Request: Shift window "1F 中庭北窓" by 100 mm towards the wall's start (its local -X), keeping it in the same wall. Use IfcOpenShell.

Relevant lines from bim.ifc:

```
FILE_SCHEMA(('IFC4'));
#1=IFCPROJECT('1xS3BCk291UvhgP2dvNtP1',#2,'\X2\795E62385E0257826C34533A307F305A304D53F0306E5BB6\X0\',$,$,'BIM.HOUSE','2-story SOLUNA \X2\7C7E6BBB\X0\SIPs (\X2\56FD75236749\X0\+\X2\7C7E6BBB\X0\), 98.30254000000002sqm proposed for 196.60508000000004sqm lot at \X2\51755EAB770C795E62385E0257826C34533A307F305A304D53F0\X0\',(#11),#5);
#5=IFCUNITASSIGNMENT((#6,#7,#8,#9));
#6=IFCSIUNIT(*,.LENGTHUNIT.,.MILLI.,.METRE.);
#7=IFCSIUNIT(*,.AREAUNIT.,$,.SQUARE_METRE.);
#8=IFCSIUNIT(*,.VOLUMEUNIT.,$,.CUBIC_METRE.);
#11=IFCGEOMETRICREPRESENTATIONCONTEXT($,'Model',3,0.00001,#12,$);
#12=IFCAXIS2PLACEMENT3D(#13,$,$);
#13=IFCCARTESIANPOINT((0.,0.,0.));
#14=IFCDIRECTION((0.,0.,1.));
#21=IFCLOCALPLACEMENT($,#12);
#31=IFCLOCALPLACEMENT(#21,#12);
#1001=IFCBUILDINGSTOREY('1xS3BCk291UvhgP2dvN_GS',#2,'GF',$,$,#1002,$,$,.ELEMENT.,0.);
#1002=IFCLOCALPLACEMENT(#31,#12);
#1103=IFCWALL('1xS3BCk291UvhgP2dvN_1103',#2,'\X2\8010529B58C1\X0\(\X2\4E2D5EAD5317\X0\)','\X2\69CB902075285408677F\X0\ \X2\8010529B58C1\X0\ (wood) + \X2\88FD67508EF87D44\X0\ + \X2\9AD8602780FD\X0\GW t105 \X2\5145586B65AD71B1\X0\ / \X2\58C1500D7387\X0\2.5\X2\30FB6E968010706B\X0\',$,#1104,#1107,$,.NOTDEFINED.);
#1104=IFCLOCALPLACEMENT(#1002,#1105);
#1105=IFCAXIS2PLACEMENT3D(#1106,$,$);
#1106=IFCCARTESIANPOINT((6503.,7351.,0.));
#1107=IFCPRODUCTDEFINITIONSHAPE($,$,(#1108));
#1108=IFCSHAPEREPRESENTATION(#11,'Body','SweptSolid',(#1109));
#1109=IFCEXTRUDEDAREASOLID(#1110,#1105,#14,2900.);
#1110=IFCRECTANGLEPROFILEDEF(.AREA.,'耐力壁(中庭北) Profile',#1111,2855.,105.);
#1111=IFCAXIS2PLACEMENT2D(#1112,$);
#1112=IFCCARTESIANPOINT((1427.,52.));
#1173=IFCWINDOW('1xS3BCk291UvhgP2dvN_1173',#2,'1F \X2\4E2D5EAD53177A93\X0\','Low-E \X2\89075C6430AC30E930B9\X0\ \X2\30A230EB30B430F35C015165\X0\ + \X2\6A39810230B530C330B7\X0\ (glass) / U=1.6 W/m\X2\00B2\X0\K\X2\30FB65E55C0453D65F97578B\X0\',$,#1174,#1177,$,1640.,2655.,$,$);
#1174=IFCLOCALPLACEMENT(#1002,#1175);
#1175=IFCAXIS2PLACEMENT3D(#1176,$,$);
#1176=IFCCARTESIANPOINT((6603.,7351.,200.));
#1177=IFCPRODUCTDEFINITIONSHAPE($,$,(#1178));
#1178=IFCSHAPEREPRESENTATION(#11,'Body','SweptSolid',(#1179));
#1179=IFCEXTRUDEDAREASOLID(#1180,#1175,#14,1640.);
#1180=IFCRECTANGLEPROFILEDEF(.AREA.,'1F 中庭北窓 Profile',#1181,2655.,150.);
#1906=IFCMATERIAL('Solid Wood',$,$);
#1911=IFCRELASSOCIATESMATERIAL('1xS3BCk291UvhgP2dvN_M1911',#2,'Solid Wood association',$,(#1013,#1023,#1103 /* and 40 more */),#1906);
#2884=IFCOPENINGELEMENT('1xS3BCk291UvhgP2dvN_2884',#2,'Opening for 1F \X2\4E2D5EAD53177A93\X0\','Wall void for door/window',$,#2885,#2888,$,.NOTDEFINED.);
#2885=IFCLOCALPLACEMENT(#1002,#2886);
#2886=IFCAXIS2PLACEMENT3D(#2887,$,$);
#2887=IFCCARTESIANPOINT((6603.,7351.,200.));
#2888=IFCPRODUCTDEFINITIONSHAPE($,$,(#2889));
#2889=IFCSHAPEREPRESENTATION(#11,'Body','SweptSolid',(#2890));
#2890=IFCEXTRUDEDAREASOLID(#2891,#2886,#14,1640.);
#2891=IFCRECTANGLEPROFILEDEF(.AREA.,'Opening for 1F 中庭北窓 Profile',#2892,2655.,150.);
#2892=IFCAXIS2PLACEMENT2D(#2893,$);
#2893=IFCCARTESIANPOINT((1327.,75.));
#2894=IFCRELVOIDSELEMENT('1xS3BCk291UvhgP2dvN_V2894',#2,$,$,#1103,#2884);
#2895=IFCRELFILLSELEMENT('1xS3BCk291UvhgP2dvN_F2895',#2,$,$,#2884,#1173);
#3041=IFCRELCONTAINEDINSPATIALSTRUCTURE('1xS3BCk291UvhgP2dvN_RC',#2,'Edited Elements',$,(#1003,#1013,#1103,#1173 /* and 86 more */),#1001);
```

```python
import ifcopenshell
import ifcopenshell.api.geometry
import ifcopenshell.util.placement

model = ifcopenshell.open("bim.ifc")

window = model.by_guid("1xS3BCk291UvhgP2dvN_1173")
opening = window.FillsVoids[0].RelatingOpeningElement
wall = opening.VoidsElements[0].RelatingBuildingElement

wall_matrix = ifcopenshell.util.placement.get_local_placement(wall.ObjectPlacement)
shift = wall_matrix[:3, 0] * -100.0
before = ifcopenshell.util.placement.get_local_placement(window.ObjectPlacement)[:3, 3].copy()

# The window is not placed relative to its opening, so move both.
for product in (opening, window):
    matrix = ifcopenshell.util.placement.get_local_placement(product.ObjectPlacement)
    matrix[:3, 3] += shift
    ifcopenshell.api.geometry.edit_object_placement(model, product=product, matrix=matrix, is_si=False)

after = ifcopenshell.util.placement.get_local_placement(window.ObjectPlacement)[:3, 3]
print("window moved by", (after - before).round(3) + 0.0)

model.write("bim_rev.ifc")
```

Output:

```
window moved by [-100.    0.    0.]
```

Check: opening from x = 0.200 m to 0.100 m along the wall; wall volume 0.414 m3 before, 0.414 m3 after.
